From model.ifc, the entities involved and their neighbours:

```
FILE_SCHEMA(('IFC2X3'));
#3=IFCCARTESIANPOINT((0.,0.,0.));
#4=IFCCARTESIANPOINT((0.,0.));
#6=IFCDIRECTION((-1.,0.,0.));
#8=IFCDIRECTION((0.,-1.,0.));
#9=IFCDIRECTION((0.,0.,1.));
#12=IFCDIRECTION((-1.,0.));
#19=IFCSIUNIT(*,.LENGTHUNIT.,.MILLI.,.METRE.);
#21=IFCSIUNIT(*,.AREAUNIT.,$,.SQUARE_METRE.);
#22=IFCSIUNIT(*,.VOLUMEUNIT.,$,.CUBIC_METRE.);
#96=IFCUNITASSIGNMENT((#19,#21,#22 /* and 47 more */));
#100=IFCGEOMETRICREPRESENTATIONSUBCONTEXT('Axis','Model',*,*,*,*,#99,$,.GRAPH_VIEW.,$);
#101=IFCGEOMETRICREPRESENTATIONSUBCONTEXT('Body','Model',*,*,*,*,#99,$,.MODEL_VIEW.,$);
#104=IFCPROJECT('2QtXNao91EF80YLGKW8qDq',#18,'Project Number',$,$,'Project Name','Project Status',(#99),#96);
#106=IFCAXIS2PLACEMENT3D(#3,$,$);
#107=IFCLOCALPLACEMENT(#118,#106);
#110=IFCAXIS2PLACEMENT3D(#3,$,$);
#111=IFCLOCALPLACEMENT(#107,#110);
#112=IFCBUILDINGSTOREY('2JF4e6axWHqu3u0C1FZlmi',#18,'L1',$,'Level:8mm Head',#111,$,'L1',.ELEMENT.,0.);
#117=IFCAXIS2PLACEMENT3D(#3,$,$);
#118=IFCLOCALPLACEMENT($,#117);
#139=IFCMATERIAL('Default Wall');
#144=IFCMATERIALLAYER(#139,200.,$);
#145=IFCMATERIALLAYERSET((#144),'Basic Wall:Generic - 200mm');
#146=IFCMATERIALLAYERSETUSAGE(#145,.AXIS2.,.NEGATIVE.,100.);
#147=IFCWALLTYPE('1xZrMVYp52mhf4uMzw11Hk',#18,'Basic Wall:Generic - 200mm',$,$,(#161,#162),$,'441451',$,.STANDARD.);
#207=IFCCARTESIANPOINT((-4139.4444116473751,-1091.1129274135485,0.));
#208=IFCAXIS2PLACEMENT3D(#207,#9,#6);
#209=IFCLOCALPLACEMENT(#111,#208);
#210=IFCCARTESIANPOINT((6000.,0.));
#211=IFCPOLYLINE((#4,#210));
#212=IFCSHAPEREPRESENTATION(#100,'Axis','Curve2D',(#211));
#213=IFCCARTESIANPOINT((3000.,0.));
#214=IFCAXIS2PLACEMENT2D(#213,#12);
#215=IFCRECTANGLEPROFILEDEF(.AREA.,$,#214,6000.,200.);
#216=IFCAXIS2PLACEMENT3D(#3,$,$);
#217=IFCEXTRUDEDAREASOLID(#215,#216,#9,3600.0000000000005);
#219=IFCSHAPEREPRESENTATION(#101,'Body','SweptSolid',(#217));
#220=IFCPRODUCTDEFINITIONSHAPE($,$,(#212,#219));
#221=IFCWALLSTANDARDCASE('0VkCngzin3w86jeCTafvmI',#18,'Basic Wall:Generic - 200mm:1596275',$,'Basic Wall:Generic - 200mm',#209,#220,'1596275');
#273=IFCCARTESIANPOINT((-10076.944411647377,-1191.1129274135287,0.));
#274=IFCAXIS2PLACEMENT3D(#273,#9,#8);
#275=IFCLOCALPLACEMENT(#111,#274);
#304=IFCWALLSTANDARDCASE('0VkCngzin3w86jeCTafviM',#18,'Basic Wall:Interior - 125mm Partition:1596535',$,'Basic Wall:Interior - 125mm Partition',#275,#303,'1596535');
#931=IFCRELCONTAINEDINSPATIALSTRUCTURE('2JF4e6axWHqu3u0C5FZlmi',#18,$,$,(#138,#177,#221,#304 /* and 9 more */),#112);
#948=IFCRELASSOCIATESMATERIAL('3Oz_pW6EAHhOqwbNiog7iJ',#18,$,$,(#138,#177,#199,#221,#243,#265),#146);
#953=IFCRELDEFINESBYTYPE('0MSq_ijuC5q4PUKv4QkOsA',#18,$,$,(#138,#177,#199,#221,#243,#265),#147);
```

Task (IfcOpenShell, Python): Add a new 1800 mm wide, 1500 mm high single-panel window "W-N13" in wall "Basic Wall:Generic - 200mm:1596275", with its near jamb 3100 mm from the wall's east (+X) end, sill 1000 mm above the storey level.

```python
import numpy as np
import ifcopenshell
import ifcopenshell.api.feature
import ifcopenshell.api.geometry
import ifcopenshell.api.root
import ifcopenshell.api.spatial
import ifcopenshell.api.type
import ifcopenshell.geom
import ifcopenshell.util.element
import ifcopenshell.util.placement
import ifcopenshell.util.representation
import ifcopenshell.util.shape
import ifcopenshell.util.unit

model = ifcopenshell.open("model.ifc")
unit_scale = ifcopenshell.util.unit.calculate_unit_scale(model)
settings = ifcopenshell.geom.settings()


def volume(element):
    """Net volume in cubic metres, openings subtracted."""
    shape = ifcopenshell.geom.create_shape(settings, element)
    return ifcopenshell.util.shape.get_volume(shape.geometry)


wall = model.by_guid("0VkCngzin3w86jeCTafvmI")
storey = ifcopenshell.util.element.get_container(wall, ifc_class="IfcBuildingStorey")
context = ifcopenshell.util.representation.get_context(model, "Model", "Body", "MODEL_VIEW")
before = volume(wall)

width, height, from_end, sill = 1.8, 1.5, 3.1, 1  # metres

# The wall runs along its own X axis, and the end named is its -X end.
wall_shape = ifcopenshell.geom.create_shape(settings, wall)
x, y, z = ifcopenshell.util.shape.get_vertices(wall_shape.geometry).T
start = x.min() + from_end
face, thickness = float(y.min()), float(y.max() - y.min())
wall_matrix = ifcopenshell.util.placement.get_local_placement(wall.ObjectPlacement)
level = ifcopenshell.util.placement.get_local_placement(storey.ObjectPlacement)[2, 3]


def in_wall(x, y):
    """Placement at x, y metres in the wall's axes, at sill height."""
    matrix = wall_matrix.copy()
    matrix[:, 3] = wall_matrix @ np.array([x / unit_scale, y / unit_scale, 0.0, 1.0])
    matrix[2, 3] = level + sill / unit_scale
    return matrix


# Opening: a box that overshoots both wall faces by 50 mm.
opening = ifcopenshell.api.root.create_entity(model, ifc_class="IfcOpeningElement")
box = ifcopenshell.api.geometry.add_wall_representation(
    model, context=context, length=width, height=height, thickness=thickness + 0.1
)
ifcopenshell.api.geometry.assign_representation(model, product=opening, representation=box)
ifcopenshell.api.geometry.edit_object_placement(model, product=opening, matrix=in_wall(start, face - 0.05), is_si=False)
ifcopenshell.api.feature.add_feature(model, feature=opening, element=wall)

window = ifcopenshell.api.root.create_entity(model, ifc_class="IfcWindow", name="W-N13")
window.OverallWidth, window.OverallHeight = width / unit_scale, height / unit_scale
body = ifcopenshell.api.geometry.add_window_representation(
    model,
    context=context,
    overall_width=window.OverallWidth,
    overall_height=window.OverallHeight,
    partition_type="SINGLE_PANEL",
)
ifcopenshell.api.geometry.assign_representation(model, product=window, representation=body)
ifcopenshell.api.spatial.assign_container(model, products=[window], relating_structure=storey)
fills = ifcopenshell.api.feature.add_filling(model, opening=opening, element=window)
fills.OwnerHistory = window.OwnerHistory  # required in IFC2X3

# IFC2X3 keeps the operation on the window style.
style = ifcopenshell.api.root.create_entity(model, ifc_class="IfcWindowStyle", name="W-N13")
style.OperationType, style.ConstructionType = "SINGLE_PANEL", "NOTDEFINED"
style.ParameterTakesPrecedence = style.Sizeable = False
ifcopenshell.api.type.assign_type(model, related_objects=[window], relating_type=style)

# Centre the window in the wall's thickness.
ifcopenshell.api.geometry.edit_object_placement(model, product=window, matrix=in_wall(start, face), is_si=False)
window_shape = ifcopenshell.geom.create_shape(settings, window)
depth = ifcopenshell.util.shape.get_vertices(window_shape.geometry)[:, 1]
offset = face + thickness / 2 - (depth.min() + depth.max()) / 2
ifcopenshell.api.geometry.edit_object_placement(model, product=window, matrix=in_wall(start, offset), is_si=False)

after = volume(wall)

print(f"wall volume {before:.3f} -> {after:.3f} m3")

model.write("model_edited.ifc")
```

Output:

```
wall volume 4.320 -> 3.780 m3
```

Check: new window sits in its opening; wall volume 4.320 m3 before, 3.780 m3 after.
